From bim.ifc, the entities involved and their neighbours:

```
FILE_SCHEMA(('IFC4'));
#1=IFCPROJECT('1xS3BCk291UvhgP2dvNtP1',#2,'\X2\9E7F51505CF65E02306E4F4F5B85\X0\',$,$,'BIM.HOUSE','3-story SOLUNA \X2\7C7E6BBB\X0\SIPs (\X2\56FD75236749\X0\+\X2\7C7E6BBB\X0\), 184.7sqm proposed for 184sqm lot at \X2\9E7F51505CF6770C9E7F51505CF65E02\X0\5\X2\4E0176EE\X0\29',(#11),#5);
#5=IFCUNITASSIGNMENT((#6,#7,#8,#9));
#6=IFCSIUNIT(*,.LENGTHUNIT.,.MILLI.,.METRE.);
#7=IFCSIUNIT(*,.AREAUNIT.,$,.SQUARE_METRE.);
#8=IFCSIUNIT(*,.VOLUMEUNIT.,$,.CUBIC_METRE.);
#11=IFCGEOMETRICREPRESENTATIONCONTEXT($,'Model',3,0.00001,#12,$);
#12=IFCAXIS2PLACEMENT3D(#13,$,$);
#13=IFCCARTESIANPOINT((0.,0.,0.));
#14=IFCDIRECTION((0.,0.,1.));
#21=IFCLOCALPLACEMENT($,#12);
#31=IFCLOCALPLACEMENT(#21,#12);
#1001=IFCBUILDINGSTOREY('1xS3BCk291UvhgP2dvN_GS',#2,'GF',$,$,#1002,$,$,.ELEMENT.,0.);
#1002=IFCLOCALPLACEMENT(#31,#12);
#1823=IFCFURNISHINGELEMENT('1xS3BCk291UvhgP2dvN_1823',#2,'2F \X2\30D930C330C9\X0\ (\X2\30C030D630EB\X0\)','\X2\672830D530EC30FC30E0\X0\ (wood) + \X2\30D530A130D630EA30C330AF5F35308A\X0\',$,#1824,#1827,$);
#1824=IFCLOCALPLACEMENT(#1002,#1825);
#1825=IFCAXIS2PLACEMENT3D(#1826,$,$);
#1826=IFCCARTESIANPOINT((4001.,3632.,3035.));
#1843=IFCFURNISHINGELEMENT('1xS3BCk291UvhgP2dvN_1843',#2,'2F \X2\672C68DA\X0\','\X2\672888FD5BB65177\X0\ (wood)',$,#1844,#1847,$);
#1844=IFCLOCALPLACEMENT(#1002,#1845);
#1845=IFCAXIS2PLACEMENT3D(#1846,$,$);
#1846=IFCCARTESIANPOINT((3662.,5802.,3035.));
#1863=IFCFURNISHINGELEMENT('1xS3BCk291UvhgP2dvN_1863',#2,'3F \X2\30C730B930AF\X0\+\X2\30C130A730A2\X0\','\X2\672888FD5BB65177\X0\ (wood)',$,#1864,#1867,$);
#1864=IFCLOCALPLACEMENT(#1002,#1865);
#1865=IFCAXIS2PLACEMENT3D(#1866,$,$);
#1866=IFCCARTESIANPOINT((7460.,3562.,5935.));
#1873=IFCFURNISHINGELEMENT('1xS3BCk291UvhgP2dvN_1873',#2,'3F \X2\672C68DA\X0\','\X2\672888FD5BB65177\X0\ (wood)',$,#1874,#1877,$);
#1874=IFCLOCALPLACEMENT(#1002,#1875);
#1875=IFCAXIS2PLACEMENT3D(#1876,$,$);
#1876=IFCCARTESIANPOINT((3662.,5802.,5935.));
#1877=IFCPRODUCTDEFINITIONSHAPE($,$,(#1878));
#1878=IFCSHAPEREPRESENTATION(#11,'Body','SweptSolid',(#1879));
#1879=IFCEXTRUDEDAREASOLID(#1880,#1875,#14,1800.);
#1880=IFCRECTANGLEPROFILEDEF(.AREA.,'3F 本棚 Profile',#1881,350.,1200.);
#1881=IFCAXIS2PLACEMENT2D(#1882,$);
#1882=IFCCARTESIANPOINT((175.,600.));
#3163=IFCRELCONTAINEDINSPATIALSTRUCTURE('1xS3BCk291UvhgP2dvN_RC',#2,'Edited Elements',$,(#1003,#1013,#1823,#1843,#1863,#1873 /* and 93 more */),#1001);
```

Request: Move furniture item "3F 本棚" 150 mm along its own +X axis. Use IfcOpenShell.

```python
import ifcopenshell
import ifcopenshell.api.geometry
import ifcopenshell.util.placement
import ifcopenshell.util.unit

model = ifcopenshell.open("bim.ifc")
unit_scale = ifcopenshell.util.unit.calculate_unit_scale(model)

item = model.by_guid("1xS3BCk291UvhgP2dvN_1873")
matrix = ifcopenshell.util.placement.get_local_placement(item.ObjectPlacement)
matrix[:3, 3] += matrix[:3, 0] * 0.15 / unit_scale
ifcopenshell.api.geometry.edit_object_placement(model, product=item, matrix=matrix, is_si=False)

print(ifcopenshell.util.placement.get_local_placement(item.ObjectPlacement).round(3) + 0.0)

model.write("bim_edited.ifc")
```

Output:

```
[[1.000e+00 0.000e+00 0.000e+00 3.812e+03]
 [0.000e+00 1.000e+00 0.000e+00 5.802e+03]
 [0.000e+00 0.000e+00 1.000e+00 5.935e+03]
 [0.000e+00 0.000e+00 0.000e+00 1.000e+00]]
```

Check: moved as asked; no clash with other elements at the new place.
